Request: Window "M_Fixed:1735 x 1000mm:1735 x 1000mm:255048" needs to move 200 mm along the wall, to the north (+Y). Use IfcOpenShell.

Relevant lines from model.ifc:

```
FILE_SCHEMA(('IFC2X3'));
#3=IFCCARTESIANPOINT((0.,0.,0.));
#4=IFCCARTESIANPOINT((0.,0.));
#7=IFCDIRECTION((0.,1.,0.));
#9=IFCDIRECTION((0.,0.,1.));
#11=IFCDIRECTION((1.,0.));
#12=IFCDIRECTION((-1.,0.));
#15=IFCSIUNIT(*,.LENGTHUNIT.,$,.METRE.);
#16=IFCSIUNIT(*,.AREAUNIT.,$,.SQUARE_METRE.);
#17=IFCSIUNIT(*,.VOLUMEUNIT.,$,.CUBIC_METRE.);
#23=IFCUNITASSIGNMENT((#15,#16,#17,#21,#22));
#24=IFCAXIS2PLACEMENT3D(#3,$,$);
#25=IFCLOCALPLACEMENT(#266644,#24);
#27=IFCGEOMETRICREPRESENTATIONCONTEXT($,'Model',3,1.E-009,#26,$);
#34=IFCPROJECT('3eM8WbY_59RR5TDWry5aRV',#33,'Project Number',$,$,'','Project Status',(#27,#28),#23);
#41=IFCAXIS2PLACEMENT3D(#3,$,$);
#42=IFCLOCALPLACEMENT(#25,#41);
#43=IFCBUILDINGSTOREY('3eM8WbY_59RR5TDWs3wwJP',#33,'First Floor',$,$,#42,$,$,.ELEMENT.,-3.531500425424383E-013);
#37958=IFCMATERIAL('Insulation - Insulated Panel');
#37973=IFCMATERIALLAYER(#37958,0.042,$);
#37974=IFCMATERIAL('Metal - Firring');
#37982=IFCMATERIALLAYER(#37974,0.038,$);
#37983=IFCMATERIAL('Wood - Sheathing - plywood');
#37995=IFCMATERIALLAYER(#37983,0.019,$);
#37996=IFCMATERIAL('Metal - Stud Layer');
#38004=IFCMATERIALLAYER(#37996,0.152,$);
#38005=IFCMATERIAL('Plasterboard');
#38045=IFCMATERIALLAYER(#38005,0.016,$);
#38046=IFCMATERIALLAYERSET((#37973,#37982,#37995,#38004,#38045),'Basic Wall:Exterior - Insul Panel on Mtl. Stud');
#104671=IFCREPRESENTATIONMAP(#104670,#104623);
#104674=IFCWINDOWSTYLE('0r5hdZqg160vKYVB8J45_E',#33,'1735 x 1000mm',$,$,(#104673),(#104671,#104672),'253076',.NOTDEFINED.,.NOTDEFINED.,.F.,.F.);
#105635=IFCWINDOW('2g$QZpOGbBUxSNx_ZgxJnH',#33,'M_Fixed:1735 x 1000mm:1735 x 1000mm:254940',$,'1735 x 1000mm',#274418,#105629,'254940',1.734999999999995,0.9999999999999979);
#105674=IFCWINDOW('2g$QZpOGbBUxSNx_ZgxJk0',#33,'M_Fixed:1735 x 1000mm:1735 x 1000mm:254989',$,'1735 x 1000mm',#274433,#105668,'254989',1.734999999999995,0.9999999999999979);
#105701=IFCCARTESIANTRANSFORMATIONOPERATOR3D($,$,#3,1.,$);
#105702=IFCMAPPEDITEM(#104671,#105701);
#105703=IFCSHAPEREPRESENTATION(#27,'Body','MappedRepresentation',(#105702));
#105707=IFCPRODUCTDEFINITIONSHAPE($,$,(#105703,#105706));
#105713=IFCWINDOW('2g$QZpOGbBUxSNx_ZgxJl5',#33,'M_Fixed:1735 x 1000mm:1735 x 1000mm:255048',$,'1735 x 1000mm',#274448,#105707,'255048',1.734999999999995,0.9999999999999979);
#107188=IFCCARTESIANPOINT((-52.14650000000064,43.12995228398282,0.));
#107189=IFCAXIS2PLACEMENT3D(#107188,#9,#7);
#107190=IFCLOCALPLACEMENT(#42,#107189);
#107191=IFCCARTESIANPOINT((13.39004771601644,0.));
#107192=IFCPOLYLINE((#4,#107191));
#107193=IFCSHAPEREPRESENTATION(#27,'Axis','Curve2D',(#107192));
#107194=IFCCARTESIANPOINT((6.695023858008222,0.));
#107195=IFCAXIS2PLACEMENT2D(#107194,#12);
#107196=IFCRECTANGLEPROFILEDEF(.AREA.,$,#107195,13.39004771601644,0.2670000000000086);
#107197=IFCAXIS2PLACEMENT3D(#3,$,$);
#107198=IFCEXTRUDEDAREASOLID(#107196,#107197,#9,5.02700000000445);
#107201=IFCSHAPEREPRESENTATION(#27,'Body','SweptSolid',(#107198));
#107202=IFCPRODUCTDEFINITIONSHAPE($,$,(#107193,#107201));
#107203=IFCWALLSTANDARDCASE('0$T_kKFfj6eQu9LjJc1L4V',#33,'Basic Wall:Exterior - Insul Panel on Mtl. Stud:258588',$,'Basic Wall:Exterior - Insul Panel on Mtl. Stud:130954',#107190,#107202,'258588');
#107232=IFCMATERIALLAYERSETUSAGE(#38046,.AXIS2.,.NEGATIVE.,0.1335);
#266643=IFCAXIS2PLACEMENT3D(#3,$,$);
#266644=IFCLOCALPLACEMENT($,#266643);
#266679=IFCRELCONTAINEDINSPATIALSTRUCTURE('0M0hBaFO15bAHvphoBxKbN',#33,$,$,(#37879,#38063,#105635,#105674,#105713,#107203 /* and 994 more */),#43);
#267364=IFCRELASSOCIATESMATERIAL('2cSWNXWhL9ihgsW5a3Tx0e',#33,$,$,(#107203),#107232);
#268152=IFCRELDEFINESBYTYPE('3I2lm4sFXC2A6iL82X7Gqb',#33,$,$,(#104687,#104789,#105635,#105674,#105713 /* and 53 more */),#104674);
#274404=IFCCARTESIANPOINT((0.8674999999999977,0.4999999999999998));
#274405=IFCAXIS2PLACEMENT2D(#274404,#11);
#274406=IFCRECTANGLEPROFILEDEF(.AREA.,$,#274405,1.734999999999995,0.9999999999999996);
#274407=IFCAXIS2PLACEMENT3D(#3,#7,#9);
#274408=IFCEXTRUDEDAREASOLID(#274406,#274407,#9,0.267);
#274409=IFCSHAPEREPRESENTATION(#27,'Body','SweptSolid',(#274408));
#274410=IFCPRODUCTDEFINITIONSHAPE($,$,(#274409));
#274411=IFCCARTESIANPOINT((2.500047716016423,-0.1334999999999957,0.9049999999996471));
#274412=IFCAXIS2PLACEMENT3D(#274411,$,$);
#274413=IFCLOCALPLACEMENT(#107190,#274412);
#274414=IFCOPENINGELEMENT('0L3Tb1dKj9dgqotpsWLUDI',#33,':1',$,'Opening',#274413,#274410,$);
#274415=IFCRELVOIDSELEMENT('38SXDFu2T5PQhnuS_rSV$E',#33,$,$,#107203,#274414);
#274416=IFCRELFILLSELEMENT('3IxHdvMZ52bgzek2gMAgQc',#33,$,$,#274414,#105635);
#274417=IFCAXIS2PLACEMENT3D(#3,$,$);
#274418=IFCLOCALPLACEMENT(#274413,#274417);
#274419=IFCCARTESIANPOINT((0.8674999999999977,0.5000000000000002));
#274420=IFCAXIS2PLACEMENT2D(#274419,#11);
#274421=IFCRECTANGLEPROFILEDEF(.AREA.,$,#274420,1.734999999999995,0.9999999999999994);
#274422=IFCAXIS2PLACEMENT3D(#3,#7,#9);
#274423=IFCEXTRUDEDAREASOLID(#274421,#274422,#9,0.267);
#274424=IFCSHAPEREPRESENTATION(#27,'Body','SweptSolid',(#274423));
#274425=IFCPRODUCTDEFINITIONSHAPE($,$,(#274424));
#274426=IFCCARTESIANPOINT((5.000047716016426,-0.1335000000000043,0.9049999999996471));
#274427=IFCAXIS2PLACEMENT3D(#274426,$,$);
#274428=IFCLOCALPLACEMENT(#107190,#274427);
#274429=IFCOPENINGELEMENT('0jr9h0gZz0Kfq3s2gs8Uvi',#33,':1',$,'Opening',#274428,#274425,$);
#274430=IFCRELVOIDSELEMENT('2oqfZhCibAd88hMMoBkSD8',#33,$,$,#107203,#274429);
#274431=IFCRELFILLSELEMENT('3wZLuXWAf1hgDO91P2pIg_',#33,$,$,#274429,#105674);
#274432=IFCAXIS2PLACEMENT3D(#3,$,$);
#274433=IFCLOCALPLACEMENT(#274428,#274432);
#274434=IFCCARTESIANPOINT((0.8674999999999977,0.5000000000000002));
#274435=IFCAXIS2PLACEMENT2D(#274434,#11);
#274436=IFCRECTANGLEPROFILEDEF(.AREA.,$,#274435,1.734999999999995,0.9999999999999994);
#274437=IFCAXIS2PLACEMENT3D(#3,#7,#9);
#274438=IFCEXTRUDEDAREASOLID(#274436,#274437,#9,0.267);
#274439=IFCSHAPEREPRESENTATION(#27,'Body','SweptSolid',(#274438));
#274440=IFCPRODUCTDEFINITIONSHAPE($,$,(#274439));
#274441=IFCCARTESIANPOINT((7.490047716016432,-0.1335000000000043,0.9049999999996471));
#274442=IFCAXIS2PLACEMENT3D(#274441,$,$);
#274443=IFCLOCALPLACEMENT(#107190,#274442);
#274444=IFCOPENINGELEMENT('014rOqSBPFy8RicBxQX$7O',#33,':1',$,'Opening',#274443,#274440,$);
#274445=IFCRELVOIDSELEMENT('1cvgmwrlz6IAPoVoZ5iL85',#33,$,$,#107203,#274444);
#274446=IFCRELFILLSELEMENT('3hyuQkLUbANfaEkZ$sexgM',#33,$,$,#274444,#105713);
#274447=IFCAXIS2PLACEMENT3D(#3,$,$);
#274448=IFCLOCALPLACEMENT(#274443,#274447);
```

```python
import ifcopenshell
import ifcopenshell.api.geometry
import ifcopenshell.util.placement
import ifcopenshell.util.unit

model = ifcopenshell.open("model.ifc")
unit_scale = ifcopenshell.util.unit.calculate_unit_scale(model)

window = model.by_guid("2g$QZpOGbBUxSNx_ZgxJl5")
opening = window.FillsVoids[0].RelatingOpeningElement
wall = opening.VoidsElements[0].RelatingBuildingElement

wall_matrix = ifcopenshell.util.placement.get_local_placement(wall.ObjectPlacement)
shift = wall_matrix[:3, 0] * 0.2 / unit_scale
before = ifcopenshell.util.placement.get_local_placement(window.ObjectPlacement)[:3, 3].copy()

# The window is placed relative to its opening, so it follows when the opening moves.
matrix = ifcopenshell.util.placement.get_local_placement(opening.ObjectPlacement)
matrix[:3, 3] += shift
ifcopenshell.api.geometry.edit_object_placement(
    model, product=opening, matrix=matrix, is_si=False, should_transform_children=True
)

after = ifcopenshell.util.placement.get_local_placement(window.ObjectPlacement)[:3, 3]
print("window moved by", (after - before).round(3) + 0.0)

model.write("model_v2.ifc")
```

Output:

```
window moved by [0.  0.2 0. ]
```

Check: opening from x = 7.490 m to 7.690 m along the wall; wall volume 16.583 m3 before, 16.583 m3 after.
